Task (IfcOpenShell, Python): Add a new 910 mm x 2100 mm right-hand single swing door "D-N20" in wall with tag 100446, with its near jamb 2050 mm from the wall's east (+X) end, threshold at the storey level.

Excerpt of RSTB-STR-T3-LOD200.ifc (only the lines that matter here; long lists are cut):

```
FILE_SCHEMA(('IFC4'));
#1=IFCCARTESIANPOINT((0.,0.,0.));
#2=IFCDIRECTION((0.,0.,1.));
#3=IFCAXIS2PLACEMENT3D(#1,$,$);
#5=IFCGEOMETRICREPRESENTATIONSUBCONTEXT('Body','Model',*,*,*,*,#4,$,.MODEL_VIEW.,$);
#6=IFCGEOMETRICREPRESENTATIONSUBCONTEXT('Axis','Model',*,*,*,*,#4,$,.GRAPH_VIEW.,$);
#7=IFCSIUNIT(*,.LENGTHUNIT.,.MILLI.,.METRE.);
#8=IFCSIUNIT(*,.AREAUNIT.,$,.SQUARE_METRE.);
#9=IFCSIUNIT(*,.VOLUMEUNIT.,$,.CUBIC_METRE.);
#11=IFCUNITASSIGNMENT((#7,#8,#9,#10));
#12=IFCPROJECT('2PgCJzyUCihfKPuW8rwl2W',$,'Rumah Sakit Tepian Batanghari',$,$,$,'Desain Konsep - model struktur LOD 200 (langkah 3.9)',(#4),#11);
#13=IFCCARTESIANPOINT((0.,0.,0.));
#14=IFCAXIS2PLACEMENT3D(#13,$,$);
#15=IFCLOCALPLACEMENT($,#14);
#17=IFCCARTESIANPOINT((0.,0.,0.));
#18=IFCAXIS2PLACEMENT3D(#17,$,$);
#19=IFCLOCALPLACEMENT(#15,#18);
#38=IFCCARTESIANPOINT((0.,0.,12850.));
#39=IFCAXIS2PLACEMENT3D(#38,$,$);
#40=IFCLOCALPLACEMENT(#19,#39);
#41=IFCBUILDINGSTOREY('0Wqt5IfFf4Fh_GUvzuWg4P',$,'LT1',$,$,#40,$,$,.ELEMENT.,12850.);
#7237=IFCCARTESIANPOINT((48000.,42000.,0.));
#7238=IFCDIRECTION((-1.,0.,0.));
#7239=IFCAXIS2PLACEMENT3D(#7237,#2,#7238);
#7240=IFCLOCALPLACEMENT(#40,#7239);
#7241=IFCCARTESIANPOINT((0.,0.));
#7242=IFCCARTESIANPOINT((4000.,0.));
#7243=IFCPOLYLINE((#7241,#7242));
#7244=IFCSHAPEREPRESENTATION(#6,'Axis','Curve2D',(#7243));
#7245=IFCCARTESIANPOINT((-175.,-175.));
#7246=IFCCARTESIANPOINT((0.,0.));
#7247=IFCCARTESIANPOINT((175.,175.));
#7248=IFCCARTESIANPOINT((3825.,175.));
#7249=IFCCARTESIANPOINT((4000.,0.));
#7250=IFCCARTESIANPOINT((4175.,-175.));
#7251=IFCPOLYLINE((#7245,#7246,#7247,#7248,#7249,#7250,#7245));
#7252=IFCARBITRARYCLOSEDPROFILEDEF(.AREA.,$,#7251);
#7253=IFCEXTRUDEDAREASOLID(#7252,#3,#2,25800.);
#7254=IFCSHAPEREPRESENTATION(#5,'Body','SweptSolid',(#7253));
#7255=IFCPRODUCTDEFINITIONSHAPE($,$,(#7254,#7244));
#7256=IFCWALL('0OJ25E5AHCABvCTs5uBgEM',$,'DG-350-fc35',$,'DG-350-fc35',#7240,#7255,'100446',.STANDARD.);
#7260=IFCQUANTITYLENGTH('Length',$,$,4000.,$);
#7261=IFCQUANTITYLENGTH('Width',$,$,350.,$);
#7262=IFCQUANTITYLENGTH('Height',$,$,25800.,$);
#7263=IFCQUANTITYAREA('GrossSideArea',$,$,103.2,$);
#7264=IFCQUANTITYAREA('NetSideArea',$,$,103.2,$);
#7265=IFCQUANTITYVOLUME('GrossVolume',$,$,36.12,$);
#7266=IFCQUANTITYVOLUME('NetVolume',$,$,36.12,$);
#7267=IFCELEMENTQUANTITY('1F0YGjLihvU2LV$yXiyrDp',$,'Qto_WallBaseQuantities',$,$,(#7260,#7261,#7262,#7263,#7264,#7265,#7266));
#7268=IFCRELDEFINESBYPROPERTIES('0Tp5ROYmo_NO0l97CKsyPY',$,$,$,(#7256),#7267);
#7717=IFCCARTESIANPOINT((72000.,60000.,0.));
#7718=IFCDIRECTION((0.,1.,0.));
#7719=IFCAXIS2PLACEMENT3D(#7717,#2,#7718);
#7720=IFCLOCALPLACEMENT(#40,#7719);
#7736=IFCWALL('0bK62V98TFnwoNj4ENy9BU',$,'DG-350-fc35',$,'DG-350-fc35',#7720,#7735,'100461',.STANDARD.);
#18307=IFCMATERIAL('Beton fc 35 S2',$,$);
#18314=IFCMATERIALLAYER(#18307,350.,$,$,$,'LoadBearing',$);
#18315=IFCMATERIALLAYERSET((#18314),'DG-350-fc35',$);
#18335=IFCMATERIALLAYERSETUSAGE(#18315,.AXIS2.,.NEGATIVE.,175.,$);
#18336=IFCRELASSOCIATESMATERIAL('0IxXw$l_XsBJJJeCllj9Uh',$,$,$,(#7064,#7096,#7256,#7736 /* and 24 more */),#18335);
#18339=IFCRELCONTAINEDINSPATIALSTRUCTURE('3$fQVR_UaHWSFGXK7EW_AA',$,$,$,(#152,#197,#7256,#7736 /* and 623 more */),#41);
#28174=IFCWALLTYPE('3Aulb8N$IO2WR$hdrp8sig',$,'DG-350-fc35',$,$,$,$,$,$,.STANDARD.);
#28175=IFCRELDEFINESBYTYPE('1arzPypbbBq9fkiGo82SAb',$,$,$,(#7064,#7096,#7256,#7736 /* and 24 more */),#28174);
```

```python
import numpy as np
import ifcopenshell
import ifcopenshell.api.feature
import ifcopenshell.api.geometry
import ifcopenshell.api.pset
import ifcopenshell.api.root
import ifcopenshell.api.spatial
import ifcopenshell.geom
import ifcopenshell.util.element
import ifcopenshell.util.placement
import ifcopenshell.util.representation
import ifcopenshell.util.shape
import ifcopenshell.util.unit

model = ifcopenshell.open("RSTB-STR-T3-LOD200.ifc")
unit_scale = ifcopenshell.util.unit.calculate_unit_scale(model)
area_scale = ifcopenshell.util.unit.calculate_unit_scale(model, "AREAUNIT")
volume_scale = ifcopenshell.util.unit.calculate_unit_scale(model, "VOLUMEUNIT")
settings = ifcopenshell.geom.settings()


def volume(element):
    """Net volume in cubic metres, openings subtracted."""
    shape = ifcopenshell.geom.create_shape(settings, element)
    return ifcopenshell.util.shape.get_volume(shape.geometry)


wall = model.by_id(7256)
storey = ifcopenshell.util.element.get_container(wall, ifc_class="IfcBuildingStorey")
context = ifcopenshell.util.representation.get_context(model, "Model", "Body", "MODEL_VIEW")
before = volume(wall)

width, height, from_end, sill = 0.91, 2.1, 2.05, 0.0  # metres

# The wall runs along its own X axis, and the end named is its -X end.
wall_shape = ifcopenshell.geom.create_shape(settings, wall)
x, y, z = ifcopenshell.util.shape.get_vertices(wall_shape.geometry).T
start = x.min() + from_end
face, thickness = float(y.min()), float(y.max() - y.min())
wall_matrix = ifcopenshell.util.placement.get_local_placement(wall.ObjectPlacement)
level = ifcopenshell.util.placement.get_local_placement(storey.ObjectPlacement)[2, 3]


def in_wall(x, y):
    """Placement at x, y metres in the wall's axes, at sill height."""
    matrix = wall_matrix.copy()
    matrix[:, 3] = wall_matrix @ np.array([x / unit_scale, y / unit_scale, 0.0, 1.0])
    matrix[2, 3] = level + sill / unit_scale
    return matrix


# Opening: a box that overshoots both wall faces by 50 mm.
opening = ifcopenshell.api.root.create_entity(model, ifc_class="IfcOpeningElement", predefined_type="OPENING")
box = ifcopenshell.api.geometry.add_wall_representation(
    model, context=context, length=width, height=height, thickness=thickness + 0.1
)
ifcopenshell.api.geometry.assign_representation(model, product=opening, representation=box)
ifcopenshell.api.geometry.edit_object_placement(model, product=opening, matrix=in_wall(start, face - 0.05), is_si=False)
ifcopenshell.api.feature.add_feature(model, feature=opening, element=wall)

door = ifcopenshell.api.root.create_entity(model, ifc_class="IfcDoor", name="D-N20", predefined_type="DOOR")
door.OverallWidth, door.OverallHeight = width / unit_scale, height / unit_scale
door.OperationType = "SINGLE_SWING_RIGHT"
body = ifcopenshell.api.geometry.add_door_representation(
    model,
    context=context,
    overall_width=door.OverallWidth,
    overall_height=door.OverallHeight,
    operation_type="SINGLE_SWING_RIGHT",
    lining_properties={"LiningDepth": thickness / unit_scale, "ThresholdDepth": thickness / unit_scale},
)
ifcopenshell.api.geometry.assign_representation(model, product=door, representation=body)
ifcopenshell.api.spatial.assign_container(model, products=[door], relating_structure=storey)
ifcopenshell.api.feature.add_filling(model, opening=opening, element=door)

# The lining spans the wall, so the door starts at the wall face.
ifcopenshell.api.geometry.edit_object_placement(model, product=door, matrix=in_wall(start, face), is_si=False)

after = volume(wall)

# Update the wall's stored quantities.
qto = model.by_id(ifcopenshell.util.element.get_pset(wall, "Qto_WallBaseQuantities", should_inherit=False)["id"])
ifcopenshell.api.pset.edit_qto(model, qto=qto, properties={
    "NetSideArea": after / thickness / area_scale,
    "NetVolume": after / volume_scale,
})

print(f"wall volume {before:.3f} -> {after:.3f} m3")

model.write("RSTB-STR-T3-LOD200_edited.ifc")
```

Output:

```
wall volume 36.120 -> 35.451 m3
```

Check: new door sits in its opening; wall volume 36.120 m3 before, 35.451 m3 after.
